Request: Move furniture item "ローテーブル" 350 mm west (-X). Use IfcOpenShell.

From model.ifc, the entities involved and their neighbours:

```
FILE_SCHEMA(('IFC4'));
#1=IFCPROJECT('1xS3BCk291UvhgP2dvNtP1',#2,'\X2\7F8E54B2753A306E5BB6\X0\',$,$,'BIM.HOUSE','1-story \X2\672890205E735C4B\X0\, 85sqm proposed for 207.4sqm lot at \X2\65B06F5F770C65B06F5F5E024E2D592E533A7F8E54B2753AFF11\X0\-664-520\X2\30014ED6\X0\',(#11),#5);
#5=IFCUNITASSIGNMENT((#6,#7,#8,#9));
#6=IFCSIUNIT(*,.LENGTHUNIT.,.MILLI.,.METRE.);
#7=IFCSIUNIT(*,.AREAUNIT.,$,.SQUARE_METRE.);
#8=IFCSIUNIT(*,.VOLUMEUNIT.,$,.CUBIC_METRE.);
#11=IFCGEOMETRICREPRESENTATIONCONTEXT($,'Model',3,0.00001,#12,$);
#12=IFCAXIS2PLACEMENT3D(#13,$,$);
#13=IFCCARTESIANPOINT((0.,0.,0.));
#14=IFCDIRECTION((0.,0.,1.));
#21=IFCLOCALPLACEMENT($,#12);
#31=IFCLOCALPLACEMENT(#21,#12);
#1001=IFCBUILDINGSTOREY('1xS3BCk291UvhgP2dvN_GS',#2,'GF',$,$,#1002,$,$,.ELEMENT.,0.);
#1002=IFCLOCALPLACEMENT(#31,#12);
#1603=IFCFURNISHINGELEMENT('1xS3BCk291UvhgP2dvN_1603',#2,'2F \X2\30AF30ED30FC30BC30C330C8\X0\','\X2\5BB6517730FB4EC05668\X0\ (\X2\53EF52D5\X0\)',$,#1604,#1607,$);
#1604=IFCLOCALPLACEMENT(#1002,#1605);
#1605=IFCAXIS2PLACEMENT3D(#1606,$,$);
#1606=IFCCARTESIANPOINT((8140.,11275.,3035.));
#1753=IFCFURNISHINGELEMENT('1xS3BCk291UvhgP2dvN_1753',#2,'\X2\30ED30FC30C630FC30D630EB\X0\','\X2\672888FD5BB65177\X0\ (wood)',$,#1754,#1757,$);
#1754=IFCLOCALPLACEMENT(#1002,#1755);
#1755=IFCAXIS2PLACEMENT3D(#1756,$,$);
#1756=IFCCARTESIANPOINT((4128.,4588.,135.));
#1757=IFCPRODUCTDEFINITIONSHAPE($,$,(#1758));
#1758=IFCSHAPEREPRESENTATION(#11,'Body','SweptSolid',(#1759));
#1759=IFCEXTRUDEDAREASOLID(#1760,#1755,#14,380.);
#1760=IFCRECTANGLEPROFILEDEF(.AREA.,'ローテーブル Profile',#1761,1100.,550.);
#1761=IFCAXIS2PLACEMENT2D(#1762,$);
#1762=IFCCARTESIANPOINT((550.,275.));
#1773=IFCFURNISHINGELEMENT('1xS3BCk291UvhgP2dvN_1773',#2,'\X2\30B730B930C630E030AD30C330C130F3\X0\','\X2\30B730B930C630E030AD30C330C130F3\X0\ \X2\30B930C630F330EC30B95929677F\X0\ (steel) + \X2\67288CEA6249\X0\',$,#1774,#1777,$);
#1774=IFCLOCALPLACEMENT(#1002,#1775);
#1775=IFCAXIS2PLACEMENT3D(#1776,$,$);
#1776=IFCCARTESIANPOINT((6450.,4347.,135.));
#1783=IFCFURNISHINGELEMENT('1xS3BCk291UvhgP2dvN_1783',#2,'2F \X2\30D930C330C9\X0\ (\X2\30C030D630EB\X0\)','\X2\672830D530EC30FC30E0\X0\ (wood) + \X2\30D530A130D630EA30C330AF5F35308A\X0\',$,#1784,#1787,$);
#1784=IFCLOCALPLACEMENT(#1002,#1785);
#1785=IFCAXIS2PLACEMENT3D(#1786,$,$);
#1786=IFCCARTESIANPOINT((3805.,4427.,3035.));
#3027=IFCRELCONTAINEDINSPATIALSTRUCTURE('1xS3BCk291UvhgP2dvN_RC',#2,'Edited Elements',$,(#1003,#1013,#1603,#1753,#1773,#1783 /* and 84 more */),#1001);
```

```python
import ifcopenshell
import ifcopenshell.api.geometry
import ifcopenshell.util.placement
import ifcopenshell.util.unit

model = ifcopenshell.open("model.ifc")
unit_scale = ifcopenshell.util.unit.calculate_unit_scale(model)

item = model.by_guid("1xS3BCk291UvhgP2dvN_1753")
matrix = ifcopenshell.util.placement.get_local_placement(item.ObjectPlacement)
matrix[0, 3] -= 0.35 / unit_scale
ifcopenshell.api.geometry.edit_object_placement(model, product=item, matrix=matrix, is_si=False)

print(ifcopenshell.util.placement.get_local_placement(item.ObjectPlacement).round(3) + 0.0)

model.write("model_updated.ifc")
```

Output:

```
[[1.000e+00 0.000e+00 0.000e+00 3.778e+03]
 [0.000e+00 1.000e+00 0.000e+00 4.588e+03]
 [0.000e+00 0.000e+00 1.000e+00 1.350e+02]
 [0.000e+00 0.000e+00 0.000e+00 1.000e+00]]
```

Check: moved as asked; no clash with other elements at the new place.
